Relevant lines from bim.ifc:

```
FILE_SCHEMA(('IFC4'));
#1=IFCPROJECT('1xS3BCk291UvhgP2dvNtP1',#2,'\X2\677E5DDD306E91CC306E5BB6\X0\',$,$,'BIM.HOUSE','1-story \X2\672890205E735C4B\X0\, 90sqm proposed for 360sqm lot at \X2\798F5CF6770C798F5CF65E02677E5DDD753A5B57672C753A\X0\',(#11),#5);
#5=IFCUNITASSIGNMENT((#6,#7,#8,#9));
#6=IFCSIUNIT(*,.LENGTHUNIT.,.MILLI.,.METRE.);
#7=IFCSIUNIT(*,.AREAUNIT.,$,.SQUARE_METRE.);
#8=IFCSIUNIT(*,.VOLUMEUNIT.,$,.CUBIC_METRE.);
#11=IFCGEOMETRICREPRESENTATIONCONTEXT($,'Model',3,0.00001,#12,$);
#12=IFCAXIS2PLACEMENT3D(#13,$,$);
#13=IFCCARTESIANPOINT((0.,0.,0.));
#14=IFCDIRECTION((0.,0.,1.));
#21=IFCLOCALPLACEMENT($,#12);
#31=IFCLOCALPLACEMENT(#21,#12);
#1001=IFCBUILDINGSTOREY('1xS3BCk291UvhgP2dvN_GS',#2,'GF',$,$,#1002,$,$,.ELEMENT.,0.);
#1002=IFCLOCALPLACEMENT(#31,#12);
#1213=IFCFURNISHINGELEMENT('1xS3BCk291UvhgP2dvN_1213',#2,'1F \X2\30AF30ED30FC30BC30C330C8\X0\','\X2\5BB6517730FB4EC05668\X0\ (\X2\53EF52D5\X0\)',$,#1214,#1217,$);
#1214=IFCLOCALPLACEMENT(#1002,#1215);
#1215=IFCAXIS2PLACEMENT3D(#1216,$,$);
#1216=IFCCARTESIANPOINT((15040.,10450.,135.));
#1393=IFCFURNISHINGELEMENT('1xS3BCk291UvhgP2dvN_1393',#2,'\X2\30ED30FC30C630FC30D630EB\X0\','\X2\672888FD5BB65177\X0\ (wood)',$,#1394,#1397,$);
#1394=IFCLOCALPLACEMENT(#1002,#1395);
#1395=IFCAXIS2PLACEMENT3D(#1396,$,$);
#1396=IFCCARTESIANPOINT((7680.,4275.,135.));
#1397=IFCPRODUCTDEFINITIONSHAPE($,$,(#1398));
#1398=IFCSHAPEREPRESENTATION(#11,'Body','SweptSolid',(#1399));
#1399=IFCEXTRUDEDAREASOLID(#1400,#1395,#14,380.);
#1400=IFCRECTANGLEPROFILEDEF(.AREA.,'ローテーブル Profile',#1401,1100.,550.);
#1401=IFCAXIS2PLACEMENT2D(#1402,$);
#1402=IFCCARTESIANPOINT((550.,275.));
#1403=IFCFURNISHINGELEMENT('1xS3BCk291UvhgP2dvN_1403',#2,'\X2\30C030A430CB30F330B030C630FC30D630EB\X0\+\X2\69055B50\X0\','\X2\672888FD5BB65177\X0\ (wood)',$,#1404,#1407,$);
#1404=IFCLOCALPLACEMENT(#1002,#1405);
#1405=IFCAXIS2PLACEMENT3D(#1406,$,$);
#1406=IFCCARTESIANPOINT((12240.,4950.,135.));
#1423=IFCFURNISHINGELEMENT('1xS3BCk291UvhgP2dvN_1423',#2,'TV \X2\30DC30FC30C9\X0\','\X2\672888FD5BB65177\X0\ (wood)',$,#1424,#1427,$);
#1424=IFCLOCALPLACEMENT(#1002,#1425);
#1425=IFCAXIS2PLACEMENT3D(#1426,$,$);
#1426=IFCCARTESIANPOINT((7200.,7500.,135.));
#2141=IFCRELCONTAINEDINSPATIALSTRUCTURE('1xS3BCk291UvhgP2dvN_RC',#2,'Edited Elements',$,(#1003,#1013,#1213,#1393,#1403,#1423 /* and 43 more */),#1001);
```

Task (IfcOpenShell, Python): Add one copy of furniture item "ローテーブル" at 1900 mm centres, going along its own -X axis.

```python
import ifcopenshell
import ifcopenshell.api.geometry
import ifcopenshell.api.root
import ifcopenshell.util.element
import ifcopenshell.util.placement

model = ifcopenshell.open("bim.ifc")


def reuse_history(source, copy):
    """copy_class also copies each property set's owner history, people and application; keep the originals."""
    for rel in copy.IsDefinedBy:
        if rel.is_a("IfcRelDefinesByProperties") and (history := rel.RelatingPropertyDefinition.OwnerHistory):
            rel.RelatingPropertyDefinition.OwnerHistory = source.OwnerHistory
            ifcopenshell.util.element.remove_deep2(model, history)


source = model.by_guid("1xS3BCk291UvhgP2dvN_1393")
base = ifcopenshell.util.placement.get_local_placement(source.ObjectPlacement)
step = -base[:3, 0] * 1900.0

for i in range(1, 2):
    copy = ifcopenshell.api.root.copy_class(model, product=source)
    copy.Representation = ifcopenshell.util.element.copy_deep(
        model, source.Representation, exclude=["IfcGeometricRepresentationContext", "IfcRepresentationMap"]
    )
    reuse_history(source, copy)
    matrix = base.copy()
    matrix[:3, 3] += i * step
    print("added at", matrix[:3, 3].round(3) + 0.0)
    ifcopenshell.api.geometry.edit_object_placement(model, product=copy, matrix=matrix, is_si=False)

model.write("bim_v2.ifc")
```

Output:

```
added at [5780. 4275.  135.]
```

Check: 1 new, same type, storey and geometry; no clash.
